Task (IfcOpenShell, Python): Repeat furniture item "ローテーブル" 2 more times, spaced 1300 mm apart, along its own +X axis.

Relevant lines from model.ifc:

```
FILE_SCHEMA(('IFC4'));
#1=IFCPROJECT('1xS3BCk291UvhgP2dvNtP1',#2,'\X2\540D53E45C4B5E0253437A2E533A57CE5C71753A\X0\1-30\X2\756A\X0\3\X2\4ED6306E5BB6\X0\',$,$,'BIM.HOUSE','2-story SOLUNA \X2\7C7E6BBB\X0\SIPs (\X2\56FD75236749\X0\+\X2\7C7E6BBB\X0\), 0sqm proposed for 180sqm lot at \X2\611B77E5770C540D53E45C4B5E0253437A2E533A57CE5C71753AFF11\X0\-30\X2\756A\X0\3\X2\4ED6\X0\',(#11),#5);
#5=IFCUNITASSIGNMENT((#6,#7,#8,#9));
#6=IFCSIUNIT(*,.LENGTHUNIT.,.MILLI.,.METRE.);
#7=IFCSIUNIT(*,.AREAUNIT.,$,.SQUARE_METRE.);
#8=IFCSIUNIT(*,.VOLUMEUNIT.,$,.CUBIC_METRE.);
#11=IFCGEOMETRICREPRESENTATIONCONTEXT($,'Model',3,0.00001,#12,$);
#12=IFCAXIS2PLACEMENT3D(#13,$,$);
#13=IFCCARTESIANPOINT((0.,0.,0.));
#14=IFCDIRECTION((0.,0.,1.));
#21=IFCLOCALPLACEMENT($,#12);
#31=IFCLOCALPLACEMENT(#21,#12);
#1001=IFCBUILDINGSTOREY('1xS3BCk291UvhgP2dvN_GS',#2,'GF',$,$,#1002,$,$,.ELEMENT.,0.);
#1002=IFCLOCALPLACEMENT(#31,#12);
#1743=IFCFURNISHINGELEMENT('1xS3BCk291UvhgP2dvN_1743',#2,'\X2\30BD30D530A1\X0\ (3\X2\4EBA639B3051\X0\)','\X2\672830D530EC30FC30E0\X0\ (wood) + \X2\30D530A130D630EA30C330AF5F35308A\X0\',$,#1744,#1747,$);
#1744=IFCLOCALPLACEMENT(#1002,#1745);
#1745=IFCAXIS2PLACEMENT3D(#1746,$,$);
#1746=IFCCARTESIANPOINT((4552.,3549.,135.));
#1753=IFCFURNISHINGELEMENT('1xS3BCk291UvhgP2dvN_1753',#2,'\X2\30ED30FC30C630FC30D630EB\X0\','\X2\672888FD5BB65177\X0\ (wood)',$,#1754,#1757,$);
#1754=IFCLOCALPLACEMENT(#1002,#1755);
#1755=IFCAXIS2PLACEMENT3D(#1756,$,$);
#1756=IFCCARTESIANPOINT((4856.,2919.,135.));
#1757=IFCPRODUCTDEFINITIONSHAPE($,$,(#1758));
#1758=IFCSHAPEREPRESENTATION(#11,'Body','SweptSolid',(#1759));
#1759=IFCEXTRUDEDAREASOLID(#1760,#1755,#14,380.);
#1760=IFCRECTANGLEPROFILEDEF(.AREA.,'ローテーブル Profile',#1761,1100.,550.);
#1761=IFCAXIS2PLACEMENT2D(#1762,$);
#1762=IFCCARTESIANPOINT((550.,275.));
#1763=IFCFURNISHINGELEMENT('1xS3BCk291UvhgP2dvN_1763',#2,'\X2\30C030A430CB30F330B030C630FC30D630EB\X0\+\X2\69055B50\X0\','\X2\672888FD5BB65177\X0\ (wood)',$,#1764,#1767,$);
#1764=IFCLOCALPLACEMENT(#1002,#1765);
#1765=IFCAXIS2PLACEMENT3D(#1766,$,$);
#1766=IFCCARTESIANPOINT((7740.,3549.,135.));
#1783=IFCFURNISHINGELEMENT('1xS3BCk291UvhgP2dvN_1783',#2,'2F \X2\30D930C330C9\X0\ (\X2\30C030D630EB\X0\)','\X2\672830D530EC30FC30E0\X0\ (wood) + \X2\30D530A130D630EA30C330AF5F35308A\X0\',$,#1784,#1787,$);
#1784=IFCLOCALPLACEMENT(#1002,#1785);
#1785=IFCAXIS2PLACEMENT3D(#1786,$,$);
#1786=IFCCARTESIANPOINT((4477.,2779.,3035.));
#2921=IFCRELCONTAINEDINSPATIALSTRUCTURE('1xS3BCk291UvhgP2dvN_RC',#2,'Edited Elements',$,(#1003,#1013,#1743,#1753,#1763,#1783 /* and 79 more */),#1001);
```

```python
import ifcopenshell
import ifcopenshell.api.geometry
import ifcopenshell.api.root
import ifcopenshell.util.element
import ifcopenshell.util.placement
import ifcopenshell.util.unit

model = ifcopenshell.open("model.ifc")
unit_scale = ifcopenshell.util.unit.calculate_unit_scale(model)


def reuse_history(source, copy):
    """copy_class also copies each property set's owner history, people and application; keep the originals."""
    for rel in copy.IsDefinedBy:
        if rel.is_a("IfcRelDefinesByProperties") and (history := rel.RelatingPropertyDefinition.OwnerHistory):
            rel.RelatingPropertyDefinition.OwnerHistory = source.OwnerHistory
            ifcopenshell.util.element.remove_deep2(model, history)


source = model.by_id(1753)
base = ifcopenshell.util.placement.get_local_placement(source.ObjectPlacement)
step = base[:3, 0] * 1.3 / unit_scale

for i in range(1, 3):
    copy = ifcopenshell.api.root.copy_class(model, product=source)
    copy.Representation = ifcopenshell.util.element.copy_deep(
        model, source.Representation, exclude=["IfcGeometricRepresentationContext", "IfcRepresentationMap"]
    )
    reuse_history(source, copy)
    matrix = base.copy()
    matrix[:3, 3] += i * step
    print("added at", matrix[:3, 3].round(3) + 0.0)
    ifcopenshell.api.geometry.edit_object_placement(model, product=copy, matrix=matrix, is_si=False)

model.write("model_updated.ifc")
```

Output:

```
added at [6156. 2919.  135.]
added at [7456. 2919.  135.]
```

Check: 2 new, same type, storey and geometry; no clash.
